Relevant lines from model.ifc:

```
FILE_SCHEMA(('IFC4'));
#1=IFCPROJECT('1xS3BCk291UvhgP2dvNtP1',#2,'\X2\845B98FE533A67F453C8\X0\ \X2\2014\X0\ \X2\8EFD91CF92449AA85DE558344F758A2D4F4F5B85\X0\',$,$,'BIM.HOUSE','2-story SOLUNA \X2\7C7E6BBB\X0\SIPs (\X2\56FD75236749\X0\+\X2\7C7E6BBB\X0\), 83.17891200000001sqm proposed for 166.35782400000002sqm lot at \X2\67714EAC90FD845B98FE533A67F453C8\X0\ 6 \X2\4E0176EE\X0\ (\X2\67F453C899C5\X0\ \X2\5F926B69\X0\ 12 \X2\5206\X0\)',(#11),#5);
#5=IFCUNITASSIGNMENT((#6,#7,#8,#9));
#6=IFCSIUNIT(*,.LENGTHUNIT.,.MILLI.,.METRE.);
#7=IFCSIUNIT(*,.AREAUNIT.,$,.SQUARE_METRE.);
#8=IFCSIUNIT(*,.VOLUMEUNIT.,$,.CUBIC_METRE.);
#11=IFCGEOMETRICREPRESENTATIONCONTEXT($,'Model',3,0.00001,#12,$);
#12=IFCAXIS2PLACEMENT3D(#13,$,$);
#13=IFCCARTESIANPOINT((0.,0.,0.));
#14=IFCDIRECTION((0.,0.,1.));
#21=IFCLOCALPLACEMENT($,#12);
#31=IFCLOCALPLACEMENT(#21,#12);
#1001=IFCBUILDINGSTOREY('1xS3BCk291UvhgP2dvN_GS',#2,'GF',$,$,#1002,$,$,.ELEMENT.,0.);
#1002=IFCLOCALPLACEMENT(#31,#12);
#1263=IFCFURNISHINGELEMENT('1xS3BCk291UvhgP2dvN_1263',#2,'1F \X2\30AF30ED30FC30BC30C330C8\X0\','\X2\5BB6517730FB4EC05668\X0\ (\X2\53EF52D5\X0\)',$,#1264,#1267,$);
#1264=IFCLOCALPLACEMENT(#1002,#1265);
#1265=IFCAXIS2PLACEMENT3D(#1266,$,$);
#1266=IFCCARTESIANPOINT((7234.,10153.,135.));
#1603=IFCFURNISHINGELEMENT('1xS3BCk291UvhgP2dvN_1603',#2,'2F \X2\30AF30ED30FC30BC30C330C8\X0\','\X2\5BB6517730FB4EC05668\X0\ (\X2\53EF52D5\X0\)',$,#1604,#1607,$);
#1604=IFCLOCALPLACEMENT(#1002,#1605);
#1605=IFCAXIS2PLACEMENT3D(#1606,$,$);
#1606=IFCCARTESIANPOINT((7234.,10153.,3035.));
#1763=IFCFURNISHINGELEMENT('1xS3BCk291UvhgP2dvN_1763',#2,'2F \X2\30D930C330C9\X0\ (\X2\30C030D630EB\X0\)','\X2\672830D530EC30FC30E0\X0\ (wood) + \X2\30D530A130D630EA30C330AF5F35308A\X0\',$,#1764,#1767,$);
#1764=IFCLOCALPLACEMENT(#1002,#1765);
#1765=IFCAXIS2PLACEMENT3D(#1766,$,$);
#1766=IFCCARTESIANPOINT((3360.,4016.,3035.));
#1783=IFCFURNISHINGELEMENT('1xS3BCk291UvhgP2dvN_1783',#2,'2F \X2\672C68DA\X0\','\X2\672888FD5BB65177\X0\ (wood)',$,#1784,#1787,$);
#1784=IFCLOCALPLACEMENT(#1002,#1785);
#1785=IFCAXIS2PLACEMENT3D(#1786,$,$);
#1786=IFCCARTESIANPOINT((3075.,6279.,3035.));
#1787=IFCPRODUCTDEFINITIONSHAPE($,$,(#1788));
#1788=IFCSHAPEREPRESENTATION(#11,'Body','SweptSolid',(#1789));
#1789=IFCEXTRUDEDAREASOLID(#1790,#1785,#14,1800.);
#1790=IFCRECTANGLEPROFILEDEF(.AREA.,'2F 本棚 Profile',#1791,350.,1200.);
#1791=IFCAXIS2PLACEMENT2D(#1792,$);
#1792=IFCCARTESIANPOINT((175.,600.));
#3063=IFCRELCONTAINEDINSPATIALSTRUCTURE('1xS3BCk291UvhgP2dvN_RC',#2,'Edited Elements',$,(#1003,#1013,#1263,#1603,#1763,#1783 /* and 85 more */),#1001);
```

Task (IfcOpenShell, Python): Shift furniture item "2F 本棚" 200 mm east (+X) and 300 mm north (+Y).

```python
import ifcopenshell
import ifcopenshell.api.geometry
import ifcopenshell.util.placement

model = ifcopenshell.open("model.ifc")

item = model.by_guid("1xS3BCk291UvhgP2dvN_1783")
matrix = ifcopenshell.util.placement.get_local_placement(item.ObjectPlacement)
matrix[0, 3] += 200.0
matrix[1, 3] += 300.0
ifcopenshell.api.geometry.edit_object_placement(model, product=item, matrix=matrix, is_si=False)

print(ifcopenshell.util.placement.get_local_placement(item.ObjectPlacement).round(3) + 0.0)

model.write("model_updated.ifc")
```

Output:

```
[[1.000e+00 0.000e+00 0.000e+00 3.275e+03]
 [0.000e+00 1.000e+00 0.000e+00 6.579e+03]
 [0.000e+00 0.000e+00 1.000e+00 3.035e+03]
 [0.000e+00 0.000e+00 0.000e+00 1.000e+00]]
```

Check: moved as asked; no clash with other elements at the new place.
